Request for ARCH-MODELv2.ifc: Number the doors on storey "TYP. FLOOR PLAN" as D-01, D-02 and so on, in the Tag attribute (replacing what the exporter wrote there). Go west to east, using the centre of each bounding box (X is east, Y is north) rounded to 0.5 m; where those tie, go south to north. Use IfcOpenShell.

First a look at what the model holds.

```python
import ifcopenshell
import ifcopenshell.util.element
import ifcopenshell.util.placement

model = ifcopenshell.open("ARCH-MODELv2.ifc")
print(model.schema)
storey = next(s for s in model.by_type("IfcBuildingStorey") if s.Name == "TYP. FLOOR PLAN")
doors = [e for e in ifcopenshell.util.element.get_decomposition(storey) if e.is_a("IfcDoor")]
for e in sorted(doors, key=lambda e: e.id()):
    origin = ifcopenshell.util.placement.get_local_placement(e.ObjectPlacement)[:3, 3]
    print(e.id(), e.Tag, e.Name, origin.round(2) + 0.0, sep=" | ")
```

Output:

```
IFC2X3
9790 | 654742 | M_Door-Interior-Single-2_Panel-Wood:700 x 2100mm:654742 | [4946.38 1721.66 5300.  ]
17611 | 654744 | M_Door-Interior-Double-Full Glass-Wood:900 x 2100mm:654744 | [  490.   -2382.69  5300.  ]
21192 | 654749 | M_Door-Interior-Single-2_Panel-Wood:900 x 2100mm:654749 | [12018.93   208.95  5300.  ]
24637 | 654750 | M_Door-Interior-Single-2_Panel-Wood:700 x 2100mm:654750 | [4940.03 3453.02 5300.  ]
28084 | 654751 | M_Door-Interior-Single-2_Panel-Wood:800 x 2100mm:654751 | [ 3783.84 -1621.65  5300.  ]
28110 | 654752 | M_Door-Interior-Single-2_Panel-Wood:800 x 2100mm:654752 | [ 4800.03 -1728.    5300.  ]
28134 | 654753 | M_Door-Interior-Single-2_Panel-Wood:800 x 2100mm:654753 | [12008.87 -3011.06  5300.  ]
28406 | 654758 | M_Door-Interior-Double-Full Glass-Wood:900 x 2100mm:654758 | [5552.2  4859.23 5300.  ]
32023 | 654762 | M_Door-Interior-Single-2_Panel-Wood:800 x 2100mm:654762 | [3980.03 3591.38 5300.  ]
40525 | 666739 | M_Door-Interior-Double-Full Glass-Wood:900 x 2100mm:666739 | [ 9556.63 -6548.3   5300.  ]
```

```python
import ifcopenshell
import ifcopenshell.geom
import ifcopenshell.util.element
import ifcopenshell.util.shape

model = ifcopenshell.open("ARCH-MODELv2.ifc")
settings = ifcopenshell.geom.settings()
settings.set("use-world-coords", True)


def centre(element):
    shape = ifcopenshell.geom.create_shape(settings, element)
    return ifcopenshell.util.shape.get_bbox_centroid(shape.geometry)


storey = next(s for s in model.by_type("IfcBuildingStorey") if s.Name == "TYP. FLOOR PLAN")
doors = [e for e in ifcopenshell.util.element.get_decomposition(storey) if e.is_a("IfcDoor")]

# Insertion points can sit at a corner or the storey origin, so sort by the geometry (in metres).
centres = {e: centre(e) for e in doors}
doors.sort(key=lambda e: (round(centres[e][0] / 0.5), centres[e][1]))

for i, e in enumerate(doors, start=1):
    number = f"D-{i:02d}"
    e.Tag = number
    print(e.id(), number)

model.write("ARCH-MODELv2_rev.ifc")
```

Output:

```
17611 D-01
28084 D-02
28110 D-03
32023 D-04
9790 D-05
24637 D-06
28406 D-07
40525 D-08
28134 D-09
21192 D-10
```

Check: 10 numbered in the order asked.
